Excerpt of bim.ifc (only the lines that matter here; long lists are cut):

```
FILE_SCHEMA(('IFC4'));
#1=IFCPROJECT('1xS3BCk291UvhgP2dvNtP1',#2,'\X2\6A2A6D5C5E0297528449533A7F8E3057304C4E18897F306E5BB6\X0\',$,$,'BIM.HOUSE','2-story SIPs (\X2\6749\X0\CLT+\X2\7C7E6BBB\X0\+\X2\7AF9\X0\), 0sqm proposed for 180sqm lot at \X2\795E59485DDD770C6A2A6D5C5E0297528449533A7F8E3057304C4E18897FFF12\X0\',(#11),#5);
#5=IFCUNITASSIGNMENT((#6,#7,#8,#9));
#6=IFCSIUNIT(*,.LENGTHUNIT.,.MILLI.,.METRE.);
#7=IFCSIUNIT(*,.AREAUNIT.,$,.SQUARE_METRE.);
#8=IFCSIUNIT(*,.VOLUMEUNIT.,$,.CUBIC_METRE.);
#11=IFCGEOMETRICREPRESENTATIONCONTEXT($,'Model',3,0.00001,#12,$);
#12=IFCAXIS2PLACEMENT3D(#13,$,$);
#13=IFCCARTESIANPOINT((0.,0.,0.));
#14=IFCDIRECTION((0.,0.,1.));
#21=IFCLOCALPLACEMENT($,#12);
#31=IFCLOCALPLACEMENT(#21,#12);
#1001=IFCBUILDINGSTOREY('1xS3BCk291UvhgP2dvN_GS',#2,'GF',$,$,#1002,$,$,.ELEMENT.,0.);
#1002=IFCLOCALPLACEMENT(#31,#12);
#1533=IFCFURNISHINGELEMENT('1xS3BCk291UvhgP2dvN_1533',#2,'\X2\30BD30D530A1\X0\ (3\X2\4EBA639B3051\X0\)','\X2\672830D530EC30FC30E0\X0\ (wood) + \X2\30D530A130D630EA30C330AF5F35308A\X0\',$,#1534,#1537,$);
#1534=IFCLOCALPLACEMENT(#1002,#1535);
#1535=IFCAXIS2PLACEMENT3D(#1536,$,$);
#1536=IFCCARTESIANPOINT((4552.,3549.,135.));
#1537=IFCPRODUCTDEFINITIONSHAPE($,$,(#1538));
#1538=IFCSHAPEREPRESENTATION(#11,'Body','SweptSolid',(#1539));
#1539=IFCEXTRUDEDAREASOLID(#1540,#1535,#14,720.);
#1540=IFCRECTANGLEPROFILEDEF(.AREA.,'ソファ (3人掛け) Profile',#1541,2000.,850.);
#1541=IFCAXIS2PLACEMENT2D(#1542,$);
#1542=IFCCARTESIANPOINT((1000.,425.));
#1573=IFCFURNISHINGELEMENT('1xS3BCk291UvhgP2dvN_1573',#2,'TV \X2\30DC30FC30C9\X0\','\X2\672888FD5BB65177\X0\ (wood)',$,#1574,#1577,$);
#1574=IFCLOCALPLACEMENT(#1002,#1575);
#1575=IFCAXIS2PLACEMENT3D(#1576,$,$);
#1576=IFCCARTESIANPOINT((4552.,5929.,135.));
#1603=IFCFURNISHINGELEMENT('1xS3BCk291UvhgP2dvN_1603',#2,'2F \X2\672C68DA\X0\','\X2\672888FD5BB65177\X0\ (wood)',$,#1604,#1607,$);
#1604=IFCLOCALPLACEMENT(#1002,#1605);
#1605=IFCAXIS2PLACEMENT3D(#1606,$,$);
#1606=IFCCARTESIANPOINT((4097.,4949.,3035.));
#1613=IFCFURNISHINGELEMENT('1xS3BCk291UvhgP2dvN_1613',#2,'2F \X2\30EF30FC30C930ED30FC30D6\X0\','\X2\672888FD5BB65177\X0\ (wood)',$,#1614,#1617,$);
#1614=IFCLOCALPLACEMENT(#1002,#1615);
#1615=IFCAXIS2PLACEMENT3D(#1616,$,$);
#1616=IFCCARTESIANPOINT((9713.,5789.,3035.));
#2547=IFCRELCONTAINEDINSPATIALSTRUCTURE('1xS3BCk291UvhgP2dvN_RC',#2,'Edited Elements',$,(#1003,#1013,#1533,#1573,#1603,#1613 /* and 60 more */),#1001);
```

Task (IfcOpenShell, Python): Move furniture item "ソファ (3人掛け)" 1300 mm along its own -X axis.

```python
import ifcopenshell
import ifcopenshell.api.geometry
import ifcopenshell.util.placement
import ifcopenshell.util.unit

model = ifcopenshell.open("bim.ifc")
unit_scale = ifcopenshell.util.unit.calculate_unit_scale(model)

item = model.by_guid("1xS3BCk291UvhgP2dvN_1533")
matrix = ifcopenshell.util.placement.get_local_placement(item.ObjectPlacement)
matrix[:3, 3] -= matrix[:3, 0] * 1.3 / unit_scale
ifcopenshell.api.geometry.edit_object_placement(model, product=item, matrix=matrix, is_si=False)

print(ifcopenshell.util.placement.get_local_placement(item.ObjectPlacement).round(3) + 0.0)

model.write("bim_rev.ifc")
```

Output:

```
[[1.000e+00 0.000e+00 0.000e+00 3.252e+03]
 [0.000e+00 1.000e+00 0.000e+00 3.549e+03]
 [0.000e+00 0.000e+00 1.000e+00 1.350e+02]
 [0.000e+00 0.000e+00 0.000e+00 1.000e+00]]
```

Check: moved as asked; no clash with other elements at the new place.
